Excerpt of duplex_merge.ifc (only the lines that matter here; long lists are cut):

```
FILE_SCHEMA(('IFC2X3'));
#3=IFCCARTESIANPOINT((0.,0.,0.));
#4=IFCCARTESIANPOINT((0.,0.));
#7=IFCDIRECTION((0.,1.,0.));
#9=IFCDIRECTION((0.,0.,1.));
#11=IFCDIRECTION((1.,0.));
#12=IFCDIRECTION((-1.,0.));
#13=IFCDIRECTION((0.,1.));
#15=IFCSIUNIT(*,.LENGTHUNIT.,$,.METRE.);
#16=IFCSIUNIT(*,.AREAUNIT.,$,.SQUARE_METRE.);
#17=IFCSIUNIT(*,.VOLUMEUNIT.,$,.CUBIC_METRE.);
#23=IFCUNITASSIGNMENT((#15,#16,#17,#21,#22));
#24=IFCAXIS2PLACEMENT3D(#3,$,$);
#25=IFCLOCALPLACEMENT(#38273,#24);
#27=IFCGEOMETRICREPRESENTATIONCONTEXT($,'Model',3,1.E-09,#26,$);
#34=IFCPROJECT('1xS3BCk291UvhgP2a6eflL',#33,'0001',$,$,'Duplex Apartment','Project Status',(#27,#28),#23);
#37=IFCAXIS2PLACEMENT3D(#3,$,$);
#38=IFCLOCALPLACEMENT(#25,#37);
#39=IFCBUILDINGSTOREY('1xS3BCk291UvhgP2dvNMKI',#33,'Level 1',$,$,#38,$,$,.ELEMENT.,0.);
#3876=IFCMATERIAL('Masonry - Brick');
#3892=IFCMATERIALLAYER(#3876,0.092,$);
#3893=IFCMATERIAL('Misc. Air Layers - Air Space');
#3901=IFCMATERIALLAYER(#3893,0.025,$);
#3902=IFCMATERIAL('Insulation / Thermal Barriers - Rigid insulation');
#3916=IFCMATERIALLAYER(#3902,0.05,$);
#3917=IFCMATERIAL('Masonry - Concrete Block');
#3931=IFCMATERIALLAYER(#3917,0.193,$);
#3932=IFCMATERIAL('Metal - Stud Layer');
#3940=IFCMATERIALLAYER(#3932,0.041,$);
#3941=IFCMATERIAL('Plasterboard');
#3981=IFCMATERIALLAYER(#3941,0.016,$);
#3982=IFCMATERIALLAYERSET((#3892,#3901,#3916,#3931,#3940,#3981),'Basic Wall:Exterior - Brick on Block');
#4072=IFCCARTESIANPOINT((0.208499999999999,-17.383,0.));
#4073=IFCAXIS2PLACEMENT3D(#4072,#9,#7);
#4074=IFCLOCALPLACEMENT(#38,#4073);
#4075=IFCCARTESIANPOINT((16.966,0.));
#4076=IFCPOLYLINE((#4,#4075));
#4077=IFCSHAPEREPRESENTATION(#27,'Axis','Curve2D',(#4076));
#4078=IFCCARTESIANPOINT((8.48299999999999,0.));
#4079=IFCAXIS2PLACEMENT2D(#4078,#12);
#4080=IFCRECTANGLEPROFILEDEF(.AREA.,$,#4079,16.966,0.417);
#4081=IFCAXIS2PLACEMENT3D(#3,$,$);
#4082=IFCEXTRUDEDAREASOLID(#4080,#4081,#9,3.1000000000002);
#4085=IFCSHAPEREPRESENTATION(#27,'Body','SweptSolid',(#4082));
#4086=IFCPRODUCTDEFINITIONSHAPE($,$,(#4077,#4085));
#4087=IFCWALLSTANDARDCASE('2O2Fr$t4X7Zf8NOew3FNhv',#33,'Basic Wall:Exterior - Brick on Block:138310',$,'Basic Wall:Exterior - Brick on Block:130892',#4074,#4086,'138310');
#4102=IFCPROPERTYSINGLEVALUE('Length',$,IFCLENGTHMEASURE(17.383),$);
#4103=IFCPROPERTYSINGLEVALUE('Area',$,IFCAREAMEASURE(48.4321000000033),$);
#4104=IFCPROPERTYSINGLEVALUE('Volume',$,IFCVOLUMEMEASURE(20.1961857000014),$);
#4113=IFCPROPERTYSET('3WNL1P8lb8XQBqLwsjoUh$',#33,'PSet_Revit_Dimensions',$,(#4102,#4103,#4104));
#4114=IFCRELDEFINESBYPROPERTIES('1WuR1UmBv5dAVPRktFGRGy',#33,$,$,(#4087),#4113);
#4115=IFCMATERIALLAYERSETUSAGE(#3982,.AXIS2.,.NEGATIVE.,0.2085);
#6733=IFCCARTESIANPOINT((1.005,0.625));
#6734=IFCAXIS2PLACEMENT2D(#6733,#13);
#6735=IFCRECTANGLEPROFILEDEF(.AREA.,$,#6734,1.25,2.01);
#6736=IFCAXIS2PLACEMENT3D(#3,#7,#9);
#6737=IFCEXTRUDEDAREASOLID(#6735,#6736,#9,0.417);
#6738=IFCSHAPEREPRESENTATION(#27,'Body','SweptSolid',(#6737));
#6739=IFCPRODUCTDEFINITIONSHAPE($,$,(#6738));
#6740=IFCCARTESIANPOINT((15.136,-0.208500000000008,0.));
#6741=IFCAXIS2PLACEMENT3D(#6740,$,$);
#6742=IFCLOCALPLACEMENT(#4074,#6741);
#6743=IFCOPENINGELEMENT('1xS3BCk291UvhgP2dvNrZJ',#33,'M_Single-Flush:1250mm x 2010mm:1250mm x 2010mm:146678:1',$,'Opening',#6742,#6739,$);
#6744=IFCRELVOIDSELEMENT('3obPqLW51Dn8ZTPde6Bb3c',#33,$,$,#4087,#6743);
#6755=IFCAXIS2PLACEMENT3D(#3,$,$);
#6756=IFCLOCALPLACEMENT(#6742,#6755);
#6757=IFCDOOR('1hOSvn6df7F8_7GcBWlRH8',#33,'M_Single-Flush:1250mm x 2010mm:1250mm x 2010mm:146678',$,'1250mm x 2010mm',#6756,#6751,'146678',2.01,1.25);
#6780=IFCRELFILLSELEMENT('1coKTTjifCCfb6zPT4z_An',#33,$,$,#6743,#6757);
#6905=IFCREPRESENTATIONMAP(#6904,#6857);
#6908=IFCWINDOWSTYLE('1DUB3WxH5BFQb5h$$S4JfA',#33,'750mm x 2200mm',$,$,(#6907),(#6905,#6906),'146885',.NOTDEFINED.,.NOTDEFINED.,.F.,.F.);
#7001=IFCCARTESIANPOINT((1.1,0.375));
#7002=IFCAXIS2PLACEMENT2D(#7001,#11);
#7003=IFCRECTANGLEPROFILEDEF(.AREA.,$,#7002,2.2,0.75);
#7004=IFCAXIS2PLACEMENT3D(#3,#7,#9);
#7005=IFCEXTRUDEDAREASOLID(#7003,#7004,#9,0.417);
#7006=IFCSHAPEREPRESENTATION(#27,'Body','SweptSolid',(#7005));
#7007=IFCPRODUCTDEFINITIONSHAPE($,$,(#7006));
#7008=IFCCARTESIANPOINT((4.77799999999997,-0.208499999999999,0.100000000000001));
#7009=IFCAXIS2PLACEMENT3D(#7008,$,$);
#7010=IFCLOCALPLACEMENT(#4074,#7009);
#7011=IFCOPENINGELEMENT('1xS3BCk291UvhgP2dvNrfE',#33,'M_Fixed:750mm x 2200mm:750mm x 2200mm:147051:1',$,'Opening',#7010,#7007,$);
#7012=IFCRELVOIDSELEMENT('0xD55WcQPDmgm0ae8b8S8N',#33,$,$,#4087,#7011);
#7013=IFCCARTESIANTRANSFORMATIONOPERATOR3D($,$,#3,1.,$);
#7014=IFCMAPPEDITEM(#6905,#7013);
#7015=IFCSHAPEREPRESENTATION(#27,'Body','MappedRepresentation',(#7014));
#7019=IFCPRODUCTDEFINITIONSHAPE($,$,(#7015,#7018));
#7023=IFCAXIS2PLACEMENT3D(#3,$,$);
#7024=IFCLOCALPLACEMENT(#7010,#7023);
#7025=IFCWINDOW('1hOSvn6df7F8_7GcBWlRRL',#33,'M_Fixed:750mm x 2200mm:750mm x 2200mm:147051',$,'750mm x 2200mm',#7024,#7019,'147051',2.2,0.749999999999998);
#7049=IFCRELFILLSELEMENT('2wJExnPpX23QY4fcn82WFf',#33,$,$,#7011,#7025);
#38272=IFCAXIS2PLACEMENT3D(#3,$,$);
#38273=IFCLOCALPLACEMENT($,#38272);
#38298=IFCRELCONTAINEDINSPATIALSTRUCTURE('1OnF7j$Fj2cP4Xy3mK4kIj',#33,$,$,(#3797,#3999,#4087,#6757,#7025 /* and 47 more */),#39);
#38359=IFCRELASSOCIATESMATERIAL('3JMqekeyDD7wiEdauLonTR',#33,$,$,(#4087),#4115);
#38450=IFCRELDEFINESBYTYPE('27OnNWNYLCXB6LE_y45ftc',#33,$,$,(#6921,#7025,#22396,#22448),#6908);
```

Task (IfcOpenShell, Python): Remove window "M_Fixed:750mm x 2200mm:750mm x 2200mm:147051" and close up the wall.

```python
import ifcopenshell
import ifcopenshell.api.feature
import ifcopenshell.api.pset
import ifcopenshell.api.root
import ifcopenshell.geom
import ifcopenshell.util.element
import ifcopenshell.util.shape
import ifcopenshell.util.unit

model = ifcopenshell.open("duplex_merge.ifc")
area_scale = ifcopenshell.util.unit.calculate_unit_scale(model, "AREAUNIT")
volume_scale = ifcopenshell.util.unit.calculate_unit_scale(model, "VOLUMEUNIT")
settings = ifcopenshell.geom.settings()


def volume(element):
    """Net volume in cubic metres, openings subtracted."""
    shape = ifcopenshell.geom.create_shape(settings, element)
    return ifcopenshell.util.shape.get_volume(shape.geometry)


window = model.by_guid("1hOSvn6df7F8_7GcBWlRRL")
opening = window.FillsVoids[0].RelatingOpeningElement
wall = opening.VoidsElements[0].RelatingBuildingElement
before = volume(wall)

ifcopenshell.api.root.remove_product(model, product=window)
ifcopenshell.api.feature.remove_feature(model, feature=opening)

after = volume(wall)
thickness = 0.417  # wall thickness in metres

# Update the wall's stored quantities.
pset = model.by_id(ifcopenshell.util.element.get_pset(wall, "PSet_Revit_Dimensions", should_inherit=False)["id"])
ifcopenshell.api.pset.edit_pset(model, pset=pset, properties={
    "Area": model.create_entity("IfcAreaMeasure", after / thickness / area_scale),
    "Volume": model.create_entity("IfcVolumeMeasure", after / volume_scale),
})

print(f"wall volume {before:.3f} -> {after:.3f} m3")

model.write("duplex_merge_v2.ifc")
```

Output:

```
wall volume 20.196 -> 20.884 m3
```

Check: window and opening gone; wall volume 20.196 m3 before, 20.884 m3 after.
